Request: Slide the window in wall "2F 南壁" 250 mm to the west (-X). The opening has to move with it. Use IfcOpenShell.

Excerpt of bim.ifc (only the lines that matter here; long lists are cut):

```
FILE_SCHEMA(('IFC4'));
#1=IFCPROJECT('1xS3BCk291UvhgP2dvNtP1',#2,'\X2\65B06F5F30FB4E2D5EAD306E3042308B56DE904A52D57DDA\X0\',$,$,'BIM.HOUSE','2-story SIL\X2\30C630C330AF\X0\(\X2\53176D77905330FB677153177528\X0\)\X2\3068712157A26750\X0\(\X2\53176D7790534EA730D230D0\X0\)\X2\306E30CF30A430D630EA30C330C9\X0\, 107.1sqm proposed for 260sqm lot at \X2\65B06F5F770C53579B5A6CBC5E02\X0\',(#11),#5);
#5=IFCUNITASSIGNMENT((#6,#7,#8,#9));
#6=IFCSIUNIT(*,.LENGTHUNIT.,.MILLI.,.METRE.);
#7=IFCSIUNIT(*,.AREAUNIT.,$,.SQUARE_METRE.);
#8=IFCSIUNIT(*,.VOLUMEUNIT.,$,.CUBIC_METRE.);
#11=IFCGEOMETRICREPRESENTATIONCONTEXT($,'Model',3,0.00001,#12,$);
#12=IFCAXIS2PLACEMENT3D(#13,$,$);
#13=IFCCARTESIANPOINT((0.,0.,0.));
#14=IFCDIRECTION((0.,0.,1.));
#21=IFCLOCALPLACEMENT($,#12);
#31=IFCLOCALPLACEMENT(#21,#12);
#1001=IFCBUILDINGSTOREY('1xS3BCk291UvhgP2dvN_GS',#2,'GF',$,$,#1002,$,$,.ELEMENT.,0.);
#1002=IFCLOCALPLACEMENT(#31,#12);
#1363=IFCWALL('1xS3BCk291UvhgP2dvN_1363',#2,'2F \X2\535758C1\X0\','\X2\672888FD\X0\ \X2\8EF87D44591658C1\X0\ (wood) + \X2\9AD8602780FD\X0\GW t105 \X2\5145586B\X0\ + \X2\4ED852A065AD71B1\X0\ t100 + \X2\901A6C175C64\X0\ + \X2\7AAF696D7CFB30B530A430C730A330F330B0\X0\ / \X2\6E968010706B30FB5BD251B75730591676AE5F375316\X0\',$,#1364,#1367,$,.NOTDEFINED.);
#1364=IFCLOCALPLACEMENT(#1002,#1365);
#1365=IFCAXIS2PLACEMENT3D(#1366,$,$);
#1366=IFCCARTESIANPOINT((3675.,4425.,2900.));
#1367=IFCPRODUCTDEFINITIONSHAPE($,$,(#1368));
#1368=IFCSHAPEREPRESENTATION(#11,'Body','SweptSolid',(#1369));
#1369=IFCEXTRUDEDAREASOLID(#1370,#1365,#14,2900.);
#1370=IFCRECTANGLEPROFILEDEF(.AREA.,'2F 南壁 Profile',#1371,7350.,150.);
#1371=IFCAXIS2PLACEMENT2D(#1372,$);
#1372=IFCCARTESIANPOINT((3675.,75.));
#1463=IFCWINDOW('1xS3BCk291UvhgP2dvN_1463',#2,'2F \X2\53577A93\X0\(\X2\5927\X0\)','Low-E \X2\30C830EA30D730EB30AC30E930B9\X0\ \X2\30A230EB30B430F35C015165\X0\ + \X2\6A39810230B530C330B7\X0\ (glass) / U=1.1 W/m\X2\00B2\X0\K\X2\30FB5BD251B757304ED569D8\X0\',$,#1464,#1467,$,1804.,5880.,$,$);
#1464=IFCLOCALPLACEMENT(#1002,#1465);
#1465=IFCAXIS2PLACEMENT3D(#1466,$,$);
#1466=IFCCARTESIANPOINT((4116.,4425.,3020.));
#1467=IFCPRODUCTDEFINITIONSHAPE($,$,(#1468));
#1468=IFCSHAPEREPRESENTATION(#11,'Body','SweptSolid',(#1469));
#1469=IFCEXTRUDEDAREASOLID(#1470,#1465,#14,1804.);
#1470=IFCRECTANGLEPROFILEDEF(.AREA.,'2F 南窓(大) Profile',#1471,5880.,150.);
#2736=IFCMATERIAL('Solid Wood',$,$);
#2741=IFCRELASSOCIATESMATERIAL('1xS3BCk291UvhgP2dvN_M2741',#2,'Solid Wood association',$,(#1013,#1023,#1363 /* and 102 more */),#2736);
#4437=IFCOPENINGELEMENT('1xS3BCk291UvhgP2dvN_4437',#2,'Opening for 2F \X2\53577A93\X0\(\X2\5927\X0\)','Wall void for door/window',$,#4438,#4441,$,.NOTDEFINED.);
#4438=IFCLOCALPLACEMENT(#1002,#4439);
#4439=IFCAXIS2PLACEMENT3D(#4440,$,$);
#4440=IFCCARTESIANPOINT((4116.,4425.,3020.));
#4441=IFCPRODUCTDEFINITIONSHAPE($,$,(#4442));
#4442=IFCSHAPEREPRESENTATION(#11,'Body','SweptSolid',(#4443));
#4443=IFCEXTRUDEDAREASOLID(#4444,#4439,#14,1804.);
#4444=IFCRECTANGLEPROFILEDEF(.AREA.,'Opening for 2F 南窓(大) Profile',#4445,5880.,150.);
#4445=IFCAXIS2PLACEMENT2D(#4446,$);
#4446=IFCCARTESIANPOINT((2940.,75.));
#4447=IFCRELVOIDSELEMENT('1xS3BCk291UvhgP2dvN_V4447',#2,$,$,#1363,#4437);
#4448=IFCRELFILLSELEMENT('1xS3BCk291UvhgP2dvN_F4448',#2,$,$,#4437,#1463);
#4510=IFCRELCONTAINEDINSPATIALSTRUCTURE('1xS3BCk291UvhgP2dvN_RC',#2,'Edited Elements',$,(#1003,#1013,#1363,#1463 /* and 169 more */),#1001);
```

```python
import ifcopenshell
import ifcopenshell.api.geometry
import ifcopenshell.util.placement

model = ifcopenshell.open("bim.ifc")

window = model.by_guid("1xS3BCk291UvhgP2dvN_1463")
opening = window.FillsVoids[0].RelatingOpeningElement
wall = opening.VoidsElements[0].RelatingBuildingElement

wall_matrix = ifcopenshell.util.placement.get_local_placement(wall.ObjectPlacement)
shift = wall_matrix[:3, 0] * -250.0
before = ifcopenshell.util.placement.get_local_placement(window.ObjectPlacement)[:3, 3].copy()

# The window is not placed relative to its opening, so move both.
for product in (opening, window):
    matrix = ifcopenshell.util.placement.get_local_placement(product.ObjectPlacement)
    matrix[:3, 3] += shift
    ifcopenshell.api.geometry.edit_object_placement(model, product=product, matrix=matrix, is_si=False)

after = ifcopenshell.util.placement.get_local_placement(window.ObjectPlacement)[:3, 3]
print("window moved by", (after - before).round(3) + 0.0)

model.write("bim_v2.ifc")
```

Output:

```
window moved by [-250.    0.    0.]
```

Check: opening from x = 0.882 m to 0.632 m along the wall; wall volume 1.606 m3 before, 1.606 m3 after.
